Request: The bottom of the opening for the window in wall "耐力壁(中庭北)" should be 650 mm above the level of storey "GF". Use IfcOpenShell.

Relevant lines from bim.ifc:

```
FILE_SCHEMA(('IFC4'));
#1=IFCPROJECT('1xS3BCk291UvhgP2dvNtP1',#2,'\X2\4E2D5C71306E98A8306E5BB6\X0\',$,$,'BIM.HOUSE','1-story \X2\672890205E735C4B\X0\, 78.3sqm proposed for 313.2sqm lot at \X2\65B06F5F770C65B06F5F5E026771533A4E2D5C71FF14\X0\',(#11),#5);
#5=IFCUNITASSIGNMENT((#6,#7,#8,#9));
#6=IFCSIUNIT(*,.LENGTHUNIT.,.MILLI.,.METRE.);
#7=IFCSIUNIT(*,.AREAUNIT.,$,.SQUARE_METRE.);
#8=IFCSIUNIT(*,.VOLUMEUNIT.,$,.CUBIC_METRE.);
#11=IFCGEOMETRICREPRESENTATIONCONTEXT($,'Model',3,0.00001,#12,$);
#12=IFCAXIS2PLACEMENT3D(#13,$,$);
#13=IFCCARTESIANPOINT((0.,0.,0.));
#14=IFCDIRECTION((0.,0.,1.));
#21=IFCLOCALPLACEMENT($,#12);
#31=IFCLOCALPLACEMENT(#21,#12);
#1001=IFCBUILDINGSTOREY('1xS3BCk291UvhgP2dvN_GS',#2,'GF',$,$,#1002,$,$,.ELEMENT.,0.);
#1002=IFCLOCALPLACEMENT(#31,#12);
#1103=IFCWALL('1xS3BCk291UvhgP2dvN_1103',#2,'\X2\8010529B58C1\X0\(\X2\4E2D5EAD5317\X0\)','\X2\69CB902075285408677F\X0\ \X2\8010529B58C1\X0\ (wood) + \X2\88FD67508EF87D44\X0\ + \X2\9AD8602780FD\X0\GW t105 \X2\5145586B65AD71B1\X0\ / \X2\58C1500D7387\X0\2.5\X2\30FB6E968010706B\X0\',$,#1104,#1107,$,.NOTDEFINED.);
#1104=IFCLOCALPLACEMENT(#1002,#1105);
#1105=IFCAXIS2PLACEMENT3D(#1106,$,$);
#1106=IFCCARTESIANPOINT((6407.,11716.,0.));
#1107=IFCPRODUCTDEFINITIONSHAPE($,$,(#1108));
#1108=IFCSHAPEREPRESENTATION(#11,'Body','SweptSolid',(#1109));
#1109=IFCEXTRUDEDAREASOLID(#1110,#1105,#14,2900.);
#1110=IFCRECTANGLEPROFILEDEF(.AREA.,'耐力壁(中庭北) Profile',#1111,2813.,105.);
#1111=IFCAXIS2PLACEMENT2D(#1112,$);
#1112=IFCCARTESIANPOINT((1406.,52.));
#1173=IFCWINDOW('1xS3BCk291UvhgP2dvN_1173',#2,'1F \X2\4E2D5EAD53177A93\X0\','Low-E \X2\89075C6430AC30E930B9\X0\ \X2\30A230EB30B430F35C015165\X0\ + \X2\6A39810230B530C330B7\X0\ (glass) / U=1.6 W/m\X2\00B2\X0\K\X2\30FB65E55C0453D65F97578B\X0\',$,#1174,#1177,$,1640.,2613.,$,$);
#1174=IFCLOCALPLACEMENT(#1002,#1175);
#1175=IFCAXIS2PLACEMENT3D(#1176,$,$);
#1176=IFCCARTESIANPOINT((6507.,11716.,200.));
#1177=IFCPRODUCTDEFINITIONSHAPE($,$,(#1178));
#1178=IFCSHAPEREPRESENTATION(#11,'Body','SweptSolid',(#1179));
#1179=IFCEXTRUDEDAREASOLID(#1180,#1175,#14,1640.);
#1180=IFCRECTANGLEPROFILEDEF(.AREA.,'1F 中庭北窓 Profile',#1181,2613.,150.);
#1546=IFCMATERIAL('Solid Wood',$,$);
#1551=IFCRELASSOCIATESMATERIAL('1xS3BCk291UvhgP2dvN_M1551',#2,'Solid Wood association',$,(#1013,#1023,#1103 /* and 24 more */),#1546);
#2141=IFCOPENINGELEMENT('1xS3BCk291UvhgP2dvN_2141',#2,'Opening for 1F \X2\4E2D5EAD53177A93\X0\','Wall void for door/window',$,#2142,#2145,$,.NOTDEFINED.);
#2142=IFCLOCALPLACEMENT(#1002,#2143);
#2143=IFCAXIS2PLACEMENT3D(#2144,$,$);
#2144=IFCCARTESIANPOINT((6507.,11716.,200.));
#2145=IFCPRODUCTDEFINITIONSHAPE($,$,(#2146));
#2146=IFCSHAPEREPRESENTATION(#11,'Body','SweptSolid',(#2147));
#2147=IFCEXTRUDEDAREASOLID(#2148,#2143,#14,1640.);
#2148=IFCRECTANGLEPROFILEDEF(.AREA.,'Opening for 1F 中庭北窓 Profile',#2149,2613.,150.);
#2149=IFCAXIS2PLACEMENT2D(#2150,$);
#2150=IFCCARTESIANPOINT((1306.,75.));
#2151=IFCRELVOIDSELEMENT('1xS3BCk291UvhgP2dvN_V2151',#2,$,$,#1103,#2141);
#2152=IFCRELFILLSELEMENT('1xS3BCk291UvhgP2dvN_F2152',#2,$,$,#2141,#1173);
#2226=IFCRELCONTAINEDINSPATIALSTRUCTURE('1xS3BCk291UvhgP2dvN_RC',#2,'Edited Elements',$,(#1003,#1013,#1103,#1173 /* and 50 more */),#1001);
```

```python
import numpy as np
import ifcopenshell
import ifcopenshell.api.geometry
import ifcopenshell.geom
import ifcopenshell.util.element
import ifcopenshell.util.placement
import ifcopenshell.util.shape
import ifcopenshell.util.unit

model = ifcopenshell.open("bim.ifc")
unit_scale = ifcopenshell.util.unit.calculate_unit_scale(model)

window = model.by_guid("1xS3BCk291UvhgP2dvN_1173")
opening = window.FillsVoids[0].RelatingOpeningElement
storey = ifcopenshell.util.element.get_container(window, ifc_class="IfcBuildingStorey")
level = ifcopenshell.util.placement.get_local_placement(storey.ObjectPlacement)[2, 3]

# The opening's origin need not be at the sill, so measure its lowest point.
shape = ifcopenshell.geom.create_shape(ifcopenshell.geom.settings(), opening)
bottom = ifcopenshell.util.shape.get_shape_bottom_elevation(shape, shape.geometry) / unit_scale
dz = level + 0.65 / unit_scale - bottom

shift = np.array([0.0, 0.0, dz])
# The window is not placed relative to its opening, so move both.
for product in (opening, window):
    matrix = ifcopenshell.util.placement.get_local_placement(product.ObjectPlacement)
    matrix[:3, 3] += shift
    ifcopenshell.api.geometry.edit_object_placement(model, product=product, matrix=matrix, is_si=False)

print(f"moved by {dz * unit_scale:+.3f} m")

model.write("bim_edited.ifc")
```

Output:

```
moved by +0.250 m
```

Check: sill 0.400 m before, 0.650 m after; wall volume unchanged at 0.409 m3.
